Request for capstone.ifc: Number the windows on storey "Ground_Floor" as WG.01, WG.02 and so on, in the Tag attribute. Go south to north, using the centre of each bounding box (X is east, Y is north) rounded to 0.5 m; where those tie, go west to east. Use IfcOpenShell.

First a look at what the model holds.

```python
import ifcopenshell
import ifcopenshell.util.element
import ifcopenshell.util.placement

model = ifcopenshell.open("capstone.ifc")
print(model.schema)
storey = next(s for s in model.by_type("IfcBuildingStorey") if s.Name == "Ground_Floor")
windows = [e for e in ifcopenshell.util.element.get_decomposition(storey) if e.is_a("IfcWindow")]
for e in sorted(windows, key=lambda e: e.id()):
    origin = ifcopenshell.util.placement.get_local_placement(e.ObjectPlacement)[:3, 3]
    print(e.id(), e.Tag, e.Name, origin.round(2) + 0.0, sep=" | ")
```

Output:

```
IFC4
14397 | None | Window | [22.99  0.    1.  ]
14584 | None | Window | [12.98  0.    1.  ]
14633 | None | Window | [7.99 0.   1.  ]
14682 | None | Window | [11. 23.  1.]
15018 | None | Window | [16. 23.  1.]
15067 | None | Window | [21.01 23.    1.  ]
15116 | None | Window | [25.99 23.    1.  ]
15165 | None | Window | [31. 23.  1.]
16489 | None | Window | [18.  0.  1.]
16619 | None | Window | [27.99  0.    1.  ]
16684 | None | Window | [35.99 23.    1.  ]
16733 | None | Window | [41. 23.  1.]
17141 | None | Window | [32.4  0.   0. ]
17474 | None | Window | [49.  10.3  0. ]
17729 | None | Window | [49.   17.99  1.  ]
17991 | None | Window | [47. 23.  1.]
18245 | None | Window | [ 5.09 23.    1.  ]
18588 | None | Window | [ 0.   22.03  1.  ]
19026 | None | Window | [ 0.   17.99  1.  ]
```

```python
import ifcopenshell
import ifcopenshell.geom
import ifcopenshell.util.element
import ifcopenshell.util.shape

model = ifcopenshell.open("capstone.ifc")
settings = ifcopenshell.geom.settings()
settings.set("use-world-coords", True)


def centre(element):
    shape = ifcopenshell.geom.create_shape(settings, element)
    return ifcopenshell.util.shape.get_bbox_centroid(shape.geometry)


storey = next(s for s in model.by_type("IfcBuildingStorey") if s.Name == "Ground_Floor")
windows = [e for e in ifcopenshell.util.element.get_decomposition(storey) if e.is_a("IfcWindow")]

# Insertion points can sit at a corner or the storey origin, so sort by the geometry (in metres).
centres = {e: centre(e) for e in windows}
windows.sort(key=lambda e: (round(centres[e][1] / 0.5), centres[e][0]))

for i, e in enumerate(windows, start=1):
    number = f"WG.{i:02d}"
    e.Tag = number
    print(e.id(), number)

model.write("capstone_v2.ifc")
```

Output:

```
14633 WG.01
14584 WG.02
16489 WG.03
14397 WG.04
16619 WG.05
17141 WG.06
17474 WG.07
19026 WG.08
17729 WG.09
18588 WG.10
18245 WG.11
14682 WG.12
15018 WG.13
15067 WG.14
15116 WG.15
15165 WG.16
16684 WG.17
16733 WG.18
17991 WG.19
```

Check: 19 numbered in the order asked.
